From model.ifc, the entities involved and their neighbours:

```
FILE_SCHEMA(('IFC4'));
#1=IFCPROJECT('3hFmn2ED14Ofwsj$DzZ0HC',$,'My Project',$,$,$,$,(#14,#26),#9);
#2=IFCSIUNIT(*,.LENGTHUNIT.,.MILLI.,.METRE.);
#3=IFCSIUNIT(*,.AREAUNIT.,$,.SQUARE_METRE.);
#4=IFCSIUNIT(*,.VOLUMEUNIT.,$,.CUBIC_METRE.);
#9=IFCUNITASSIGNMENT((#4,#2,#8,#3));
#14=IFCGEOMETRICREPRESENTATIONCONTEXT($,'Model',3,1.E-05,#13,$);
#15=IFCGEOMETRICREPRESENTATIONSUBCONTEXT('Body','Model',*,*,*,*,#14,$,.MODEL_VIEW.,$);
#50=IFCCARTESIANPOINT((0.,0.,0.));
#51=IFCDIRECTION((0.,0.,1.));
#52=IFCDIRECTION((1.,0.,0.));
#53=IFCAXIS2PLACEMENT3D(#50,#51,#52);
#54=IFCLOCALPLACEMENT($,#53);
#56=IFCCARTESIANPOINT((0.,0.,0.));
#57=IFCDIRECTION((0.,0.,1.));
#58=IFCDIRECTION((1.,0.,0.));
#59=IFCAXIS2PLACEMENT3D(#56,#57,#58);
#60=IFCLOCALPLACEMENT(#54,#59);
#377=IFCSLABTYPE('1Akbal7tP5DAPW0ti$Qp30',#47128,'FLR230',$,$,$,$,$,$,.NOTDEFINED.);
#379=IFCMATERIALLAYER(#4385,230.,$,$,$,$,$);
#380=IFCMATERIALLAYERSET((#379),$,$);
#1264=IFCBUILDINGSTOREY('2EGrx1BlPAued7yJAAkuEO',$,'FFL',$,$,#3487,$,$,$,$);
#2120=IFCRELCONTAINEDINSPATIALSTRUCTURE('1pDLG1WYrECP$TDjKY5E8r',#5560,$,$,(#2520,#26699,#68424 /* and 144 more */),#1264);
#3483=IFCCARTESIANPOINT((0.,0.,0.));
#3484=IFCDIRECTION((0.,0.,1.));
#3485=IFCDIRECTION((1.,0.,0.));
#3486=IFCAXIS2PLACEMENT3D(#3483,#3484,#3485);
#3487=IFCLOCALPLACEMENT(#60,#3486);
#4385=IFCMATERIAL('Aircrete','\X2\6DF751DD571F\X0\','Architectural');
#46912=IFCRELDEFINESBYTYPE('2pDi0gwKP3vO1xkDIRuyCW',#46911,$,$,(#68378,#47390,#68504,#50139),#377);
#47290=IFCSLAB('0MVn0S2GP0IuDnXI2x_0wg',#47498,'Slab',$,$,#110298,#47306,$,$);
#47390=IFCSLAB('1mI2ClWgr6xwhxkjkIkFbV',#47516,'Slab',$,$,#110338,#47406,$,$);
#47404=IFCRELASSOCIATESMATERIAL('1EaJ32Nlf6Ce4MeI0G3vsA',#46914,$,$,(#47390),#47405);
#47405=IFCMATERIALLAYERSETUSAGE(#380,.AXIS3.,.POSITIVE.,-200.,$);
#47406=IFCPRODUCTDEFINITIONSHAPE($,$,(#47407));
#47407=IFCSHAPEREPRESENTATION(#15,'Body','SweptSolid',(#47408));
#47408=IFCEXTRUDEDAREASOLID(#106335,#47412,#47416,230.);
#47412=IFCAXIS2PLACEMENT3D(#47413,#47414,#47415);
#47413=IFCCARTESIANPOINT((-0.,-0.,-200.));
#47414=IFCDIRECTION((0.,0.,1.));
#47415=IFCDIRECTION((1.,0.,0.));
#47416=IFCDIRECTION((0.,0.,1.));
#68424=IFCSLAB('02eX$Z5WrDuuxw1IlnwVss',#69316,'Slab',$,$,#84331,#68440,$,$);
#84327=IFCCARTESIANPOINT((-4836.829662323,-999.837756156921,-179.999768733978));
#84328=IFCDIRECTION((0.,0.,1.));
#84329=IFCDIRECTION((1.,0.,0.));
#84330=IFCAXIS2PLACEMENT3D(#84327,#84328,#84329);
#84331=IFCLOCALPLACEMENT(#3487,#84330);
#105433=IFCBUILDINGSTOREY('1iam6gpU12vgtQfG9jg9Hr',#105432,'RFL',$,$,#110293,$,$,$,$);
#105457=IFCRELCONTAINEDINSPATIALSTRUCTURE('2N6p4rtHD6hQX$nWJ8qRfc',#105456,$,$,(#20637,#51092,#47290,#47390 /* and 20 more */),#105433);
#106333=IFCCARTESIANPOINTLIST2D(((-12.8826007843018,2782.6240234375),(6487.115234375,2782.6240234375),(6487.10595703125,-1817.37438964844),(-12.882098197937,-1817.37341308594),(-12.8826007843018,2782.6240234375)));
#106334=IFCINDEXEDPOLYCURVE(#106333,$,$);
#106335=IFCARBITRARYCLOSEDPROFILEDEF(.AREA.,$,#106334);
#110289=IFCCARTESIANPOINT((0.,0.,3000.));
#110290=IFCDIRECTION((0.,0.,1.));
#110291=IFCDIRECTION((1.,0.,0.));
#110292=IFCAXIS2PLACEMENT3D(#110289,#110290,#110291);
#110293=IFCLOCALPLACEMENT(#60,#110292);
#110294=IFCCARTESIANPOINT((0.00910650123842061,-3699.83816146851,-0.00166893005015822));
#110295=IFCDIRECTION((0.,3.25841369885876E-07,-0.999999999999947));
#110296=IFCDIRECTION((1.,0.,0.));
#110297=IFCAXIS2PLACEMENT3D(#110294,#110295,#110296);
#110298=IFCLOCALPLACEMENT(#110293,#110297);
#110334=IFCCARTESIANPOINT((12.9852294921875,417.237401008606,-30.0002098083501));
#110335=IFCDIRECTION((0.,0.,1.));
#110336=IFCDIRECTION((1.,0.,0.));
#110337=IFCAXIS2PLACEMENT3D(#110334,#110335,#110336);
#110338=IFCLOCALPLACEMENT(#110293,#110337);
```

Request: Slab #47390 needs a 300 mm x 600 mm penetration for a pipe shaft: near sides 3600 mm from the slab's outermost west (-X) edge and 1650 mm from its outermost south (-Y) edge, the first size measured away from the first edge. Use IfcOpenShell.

```python
import numpy as np
import ifcopenshell
import ifcopenshell.api.feature
import ifcopenshell.api.geometry
import ifcopenshell.api.root
import ifcopenshell.geom
import ifcopenshell.util.placement
import ifcopenshell.util.representation
import ifcopenshell.util.shape
import ifcopenshell.util.unit

model = ifcopenshell.open("model.ifc")
unit_scale = ifcopenshell.util.unit.calculate_unit_scale(model)
settings = ifcopenshell.geom.settings()


def volume(element):
    """Net volume in cubic metres, openings subtracted."""
    shape = ifcopenshell.geom.create_shape(settings, element)
    return ifcopenshell.util.shape.get_volume(shape.geometry)


slab = model.by_guid("1mI2ClWgr6xwhxkjkIkFbV")
before = volume(slab)

# Extent in the slab's own axes, in metres. The edges named are its -X and -Y sides.
slab_shape = ifcopenshell.geom.create_shape(settings, slab)
vertices = ifcopenshell.util.shape.get_vertices(slab_shape.geometry)
x_min, y_min, bottom = vertices.min(axis=0)
top = vertices[:, 2].max()

opening = ifcopenshell.api.root.create_entity(model, ifc_class="IfcOpeningElement", name="Pipe shaft opening", predefined_type="OPENING")
context = ifcopenshell.util.representation.get_context(model, "Model", "Body", "MODEL_VIEW")
width, depth = 0.3, 0.6
outline = [(0.0, 0.0), (width, 0.0), (width, depth), (0.0, depth), (0.0, 0.0)]
# Overshoot both faces by 50 mm so the cut is clean.
shape = ifcopenshell.api.geometry.add_slab_representation(
    model, context=context, depth=top - bottom + 0.1, polyline=outline
)
ifcopenshell.api.geometry.assign_representation(model, product=opening, representation=shape)

matrix = ifcopenshell.util.placement.get_local_placement(slab.ObjectPlacement)
matrix[:, 3] = matrix @ np.append(np.array([x_min + 3.6, y_min + 1.65, bottom - 0.05]) / unit_scale, 1.0)
ifcopenshell.api.geometry.edit_object_placement(model, product=opening, matrix=matrix, is_si=False)
ifcopenshell.api.feature.add_feature(model, feature=opening, element=slab)

after = volume(slab)

print(f"slab volume {before:.3f} -> {after:.3f} m3")

model.write("model_updated.ifc")
```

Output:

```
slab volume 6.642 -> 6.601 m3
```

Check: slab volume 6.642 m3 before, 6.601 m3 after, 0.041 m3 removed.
